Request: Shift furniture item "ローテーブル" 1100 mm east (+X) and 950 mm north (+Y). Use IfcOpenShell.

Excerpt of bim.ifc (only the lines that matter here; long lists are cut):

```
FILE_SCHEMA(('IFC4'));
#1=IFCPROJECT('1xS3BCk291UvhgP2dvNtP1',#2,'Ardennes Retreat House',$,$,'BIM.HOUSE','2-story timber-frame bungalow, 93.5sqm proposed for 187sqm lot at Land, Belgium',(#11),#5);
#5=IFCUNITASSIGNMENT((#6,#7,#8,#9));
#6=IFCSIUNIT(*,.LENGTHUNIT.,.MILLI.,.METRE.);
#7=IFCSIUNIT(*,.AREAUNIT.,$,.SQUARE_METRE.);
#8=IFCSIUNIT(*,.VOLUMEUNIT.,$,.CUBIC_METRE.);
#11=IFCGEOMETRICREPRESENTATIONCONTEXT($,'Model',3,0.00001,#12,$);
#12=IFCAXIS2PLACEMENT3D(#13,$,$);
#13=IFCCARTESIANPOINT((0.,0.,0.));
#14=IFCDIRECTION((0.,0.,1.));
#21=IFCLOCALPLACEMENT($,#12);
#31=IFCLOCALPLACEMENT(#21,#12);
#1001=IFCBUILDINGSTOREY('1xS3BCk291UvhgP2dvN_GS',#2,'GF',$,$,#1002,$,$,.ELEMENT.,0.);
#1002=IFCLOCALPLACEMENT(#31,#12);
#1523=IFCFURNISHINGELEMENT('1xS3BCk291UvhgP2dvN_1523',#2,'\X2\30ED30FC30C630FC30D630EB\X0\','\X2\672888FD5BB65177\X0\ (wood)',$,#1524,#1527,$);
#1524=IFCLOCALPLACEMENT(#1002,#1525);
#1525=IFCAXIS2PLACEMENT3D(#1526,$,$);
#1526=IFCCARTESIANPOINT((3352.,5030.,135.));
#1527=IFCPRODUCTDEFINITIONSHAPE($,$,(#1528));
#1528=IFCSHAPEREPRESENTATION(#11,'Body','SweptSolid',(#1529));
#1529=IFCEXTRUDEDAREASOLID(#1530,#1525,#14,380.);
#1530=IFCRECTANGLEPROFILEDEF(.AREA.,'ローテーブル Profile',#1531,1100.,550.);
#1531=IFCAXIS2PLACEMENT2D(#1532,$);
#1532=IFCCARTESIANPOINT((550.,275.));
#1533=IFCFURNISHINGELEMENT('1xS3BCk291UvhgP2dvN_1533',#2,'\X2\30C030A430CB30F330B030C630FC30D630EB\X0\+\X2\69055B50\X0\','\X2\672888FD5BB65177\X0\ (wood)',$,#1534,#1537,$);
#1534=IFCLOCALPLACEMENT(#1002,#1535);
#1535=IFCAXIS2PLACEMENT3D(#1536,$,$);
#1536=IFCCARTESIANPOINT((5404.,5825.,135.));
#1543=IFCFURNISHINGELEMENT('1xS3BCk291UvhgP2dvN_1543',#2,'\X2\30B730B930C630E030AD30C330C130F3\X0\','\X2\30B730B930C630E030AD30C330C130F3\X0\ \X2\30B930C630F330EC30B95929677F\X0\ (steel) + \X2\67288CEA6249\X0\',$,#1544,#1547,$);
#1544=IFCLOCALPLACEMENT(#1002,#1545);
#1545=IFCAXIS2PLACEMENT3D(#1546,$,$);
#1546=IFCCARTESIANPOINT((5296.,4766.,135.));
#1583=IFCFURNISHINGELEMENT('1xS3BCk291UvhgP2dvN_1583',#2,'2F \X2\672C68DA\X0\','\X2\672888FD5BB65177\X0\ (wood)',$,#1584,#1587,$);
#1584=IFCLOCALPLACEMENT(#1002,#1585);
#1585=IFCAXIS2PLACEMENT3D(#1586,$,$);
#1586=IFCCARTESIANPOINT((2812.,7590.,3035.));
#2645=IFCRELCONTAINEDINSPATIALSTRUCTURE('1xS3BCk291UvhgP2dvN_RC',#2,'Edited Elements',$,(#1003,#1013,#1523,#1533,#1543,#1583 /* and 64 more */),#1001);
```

```python
import ifcopenshell
import ifcopenshell.api.geometry
import ifcopenshell.util.placement
import ifcopenshell.util.unit

model = ifcopenshell.open("bim.ifc")
unit_scale = ifcopenshell.util.unit.calculate_unit_scale(model)

item = model.by_guid("1xS3BCk291UvhgP2dvN_1523")
matrix = ifcopenshell.util.placement.get_local_placement(item.ObjectPlacement)
matrix[0, 3] += 1.1 / unit_scale
matrix[1, 3] += 0.95 / unit_scale
ifcopenshell.api.geometry.edit_object_placement(model, product=item, matrix=matrix, is_si=False)

print(ifcopenshell.util.placement.get_local_placement(item.ObjectPlacement).round(3) + 0.0)

model.write("bim_rev.ifc")
```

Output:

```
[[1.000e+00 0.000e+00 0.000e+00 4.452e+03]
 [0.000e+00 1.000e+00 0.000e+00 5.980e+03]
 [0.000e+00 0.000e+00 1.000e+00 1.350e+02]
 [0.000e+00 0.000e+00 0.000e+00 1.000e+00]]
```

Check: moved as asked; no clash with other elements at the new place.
